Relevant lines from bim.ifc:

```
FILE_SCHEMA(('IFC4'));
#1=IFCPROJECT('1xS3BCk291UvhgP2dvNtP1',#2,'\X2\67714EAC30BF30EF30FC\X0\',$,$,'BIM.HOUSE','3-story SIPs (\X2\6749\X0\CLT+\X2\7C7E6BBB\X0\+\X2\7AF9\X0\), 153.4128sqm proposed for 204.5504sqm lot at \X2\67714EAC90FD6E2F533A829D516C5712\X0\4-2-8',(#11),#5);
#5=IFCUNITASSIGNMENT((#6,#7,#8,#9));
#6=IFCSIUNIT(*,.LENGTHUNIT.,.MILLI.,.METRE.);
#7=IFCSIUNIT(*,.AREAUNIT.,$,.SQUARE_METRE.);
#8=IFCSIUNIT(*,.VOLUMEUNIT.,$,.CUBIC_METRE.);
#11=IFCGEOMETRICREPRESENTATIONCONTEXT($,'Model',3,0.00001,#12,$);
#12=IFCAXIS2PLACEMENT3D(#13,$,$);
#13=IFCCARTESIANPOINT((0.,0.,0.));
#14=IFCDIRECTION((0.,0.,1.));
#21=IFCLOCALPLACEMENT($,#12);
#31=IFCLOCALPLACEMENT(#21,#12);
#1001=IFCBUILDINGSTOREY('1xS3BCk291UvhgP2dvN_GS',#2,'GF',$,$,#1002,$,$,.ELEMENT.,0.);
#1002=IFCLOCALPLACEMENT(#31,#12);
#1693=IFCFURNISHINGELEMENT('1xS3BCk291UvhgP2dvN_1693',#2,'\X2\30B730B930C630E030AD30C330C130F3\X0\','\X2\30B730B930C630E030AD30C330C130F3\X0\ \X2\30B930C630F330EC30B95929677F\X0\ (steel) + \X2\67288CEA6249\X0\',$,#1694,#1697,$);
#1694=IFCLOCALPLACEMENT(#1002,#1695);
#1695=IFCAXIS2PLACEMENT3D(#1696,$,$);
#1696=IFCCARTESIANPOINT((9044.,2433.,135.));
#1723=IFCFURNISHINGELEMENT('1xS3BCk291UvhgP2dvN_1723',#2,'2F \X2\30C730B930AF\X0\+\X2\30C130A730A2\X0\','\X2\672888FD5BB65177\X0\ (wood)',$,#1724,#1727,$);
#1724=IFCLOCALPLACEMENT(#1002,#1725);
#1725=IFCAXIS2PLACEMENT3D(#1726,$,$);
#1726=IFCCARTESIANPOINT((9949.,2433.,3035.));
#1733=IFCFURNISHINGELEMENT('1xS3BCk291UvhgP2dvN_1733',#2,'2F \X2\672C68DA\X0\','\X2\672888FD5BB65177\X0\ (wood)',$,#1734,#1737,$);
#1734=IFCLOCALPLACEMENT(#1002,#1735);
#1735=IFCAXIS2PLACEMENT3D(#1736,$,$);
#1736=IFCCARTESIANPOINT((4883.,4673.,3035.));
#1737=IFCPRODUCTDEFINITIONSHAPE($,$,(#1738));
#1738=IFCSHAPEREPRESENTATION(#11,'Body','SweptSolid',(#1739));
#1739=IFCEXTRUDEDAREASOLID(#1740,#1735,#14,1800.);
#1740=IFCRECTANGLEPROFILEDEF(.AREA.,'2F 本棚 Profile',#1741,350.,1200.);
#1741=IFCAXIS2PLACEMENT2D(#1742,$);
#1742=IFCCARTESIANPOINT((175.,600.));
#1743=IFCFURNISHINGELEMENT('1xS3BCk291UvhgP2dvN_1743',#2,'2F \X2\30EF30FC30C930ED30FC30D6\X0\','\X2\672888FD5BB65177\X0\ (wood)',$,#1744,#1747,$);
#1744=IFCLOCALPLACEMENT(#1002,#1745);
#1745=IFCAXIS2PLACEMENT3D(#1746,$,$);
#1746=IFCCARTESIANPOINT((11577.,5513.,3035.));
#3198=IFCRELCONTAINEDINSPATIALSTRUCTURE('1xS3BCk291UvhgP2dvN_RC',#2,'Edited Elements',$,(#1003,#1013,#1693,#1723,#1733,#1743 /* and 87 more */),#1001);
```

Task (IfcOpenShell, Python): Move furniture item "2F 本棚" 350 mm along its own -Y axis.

```python
import ifcopenshell
import ifcopenshell.api.geometry
import ifcopenshell.util.placement
import ifcopenshell.util.unit

model = ifcopenshell.open("bim.ifc")
unit_scale = ifcopenshell.util.unit.calculate_unit_scale(model)

item = model.by_guid("1xS3BCk291UvhgP2dvN_1733")
matrix = ifcopenshell.util.placement.get_local_placement(item.ObjectPlacement)
matrix[:3, 3] -= matrix[:3, 1] * 0.35 / unit_scale
ifcopenshell.api.geometry.edit_object_placement(model, product=item, matrix=matrix, is_si=False)

print(ifcopenshell.util.placement.get_local_placement(item.ObjectPlacement).round(3) + 0.0)

model.write("bim_v2.ifc")
```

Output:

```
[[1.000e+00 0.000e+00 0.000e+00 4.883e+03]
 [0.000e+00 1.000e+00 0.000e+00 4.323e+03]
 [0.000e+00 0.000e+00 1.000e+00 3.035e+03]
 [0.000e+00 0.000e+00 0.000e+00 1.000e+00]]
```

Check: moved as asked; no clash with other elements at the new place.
